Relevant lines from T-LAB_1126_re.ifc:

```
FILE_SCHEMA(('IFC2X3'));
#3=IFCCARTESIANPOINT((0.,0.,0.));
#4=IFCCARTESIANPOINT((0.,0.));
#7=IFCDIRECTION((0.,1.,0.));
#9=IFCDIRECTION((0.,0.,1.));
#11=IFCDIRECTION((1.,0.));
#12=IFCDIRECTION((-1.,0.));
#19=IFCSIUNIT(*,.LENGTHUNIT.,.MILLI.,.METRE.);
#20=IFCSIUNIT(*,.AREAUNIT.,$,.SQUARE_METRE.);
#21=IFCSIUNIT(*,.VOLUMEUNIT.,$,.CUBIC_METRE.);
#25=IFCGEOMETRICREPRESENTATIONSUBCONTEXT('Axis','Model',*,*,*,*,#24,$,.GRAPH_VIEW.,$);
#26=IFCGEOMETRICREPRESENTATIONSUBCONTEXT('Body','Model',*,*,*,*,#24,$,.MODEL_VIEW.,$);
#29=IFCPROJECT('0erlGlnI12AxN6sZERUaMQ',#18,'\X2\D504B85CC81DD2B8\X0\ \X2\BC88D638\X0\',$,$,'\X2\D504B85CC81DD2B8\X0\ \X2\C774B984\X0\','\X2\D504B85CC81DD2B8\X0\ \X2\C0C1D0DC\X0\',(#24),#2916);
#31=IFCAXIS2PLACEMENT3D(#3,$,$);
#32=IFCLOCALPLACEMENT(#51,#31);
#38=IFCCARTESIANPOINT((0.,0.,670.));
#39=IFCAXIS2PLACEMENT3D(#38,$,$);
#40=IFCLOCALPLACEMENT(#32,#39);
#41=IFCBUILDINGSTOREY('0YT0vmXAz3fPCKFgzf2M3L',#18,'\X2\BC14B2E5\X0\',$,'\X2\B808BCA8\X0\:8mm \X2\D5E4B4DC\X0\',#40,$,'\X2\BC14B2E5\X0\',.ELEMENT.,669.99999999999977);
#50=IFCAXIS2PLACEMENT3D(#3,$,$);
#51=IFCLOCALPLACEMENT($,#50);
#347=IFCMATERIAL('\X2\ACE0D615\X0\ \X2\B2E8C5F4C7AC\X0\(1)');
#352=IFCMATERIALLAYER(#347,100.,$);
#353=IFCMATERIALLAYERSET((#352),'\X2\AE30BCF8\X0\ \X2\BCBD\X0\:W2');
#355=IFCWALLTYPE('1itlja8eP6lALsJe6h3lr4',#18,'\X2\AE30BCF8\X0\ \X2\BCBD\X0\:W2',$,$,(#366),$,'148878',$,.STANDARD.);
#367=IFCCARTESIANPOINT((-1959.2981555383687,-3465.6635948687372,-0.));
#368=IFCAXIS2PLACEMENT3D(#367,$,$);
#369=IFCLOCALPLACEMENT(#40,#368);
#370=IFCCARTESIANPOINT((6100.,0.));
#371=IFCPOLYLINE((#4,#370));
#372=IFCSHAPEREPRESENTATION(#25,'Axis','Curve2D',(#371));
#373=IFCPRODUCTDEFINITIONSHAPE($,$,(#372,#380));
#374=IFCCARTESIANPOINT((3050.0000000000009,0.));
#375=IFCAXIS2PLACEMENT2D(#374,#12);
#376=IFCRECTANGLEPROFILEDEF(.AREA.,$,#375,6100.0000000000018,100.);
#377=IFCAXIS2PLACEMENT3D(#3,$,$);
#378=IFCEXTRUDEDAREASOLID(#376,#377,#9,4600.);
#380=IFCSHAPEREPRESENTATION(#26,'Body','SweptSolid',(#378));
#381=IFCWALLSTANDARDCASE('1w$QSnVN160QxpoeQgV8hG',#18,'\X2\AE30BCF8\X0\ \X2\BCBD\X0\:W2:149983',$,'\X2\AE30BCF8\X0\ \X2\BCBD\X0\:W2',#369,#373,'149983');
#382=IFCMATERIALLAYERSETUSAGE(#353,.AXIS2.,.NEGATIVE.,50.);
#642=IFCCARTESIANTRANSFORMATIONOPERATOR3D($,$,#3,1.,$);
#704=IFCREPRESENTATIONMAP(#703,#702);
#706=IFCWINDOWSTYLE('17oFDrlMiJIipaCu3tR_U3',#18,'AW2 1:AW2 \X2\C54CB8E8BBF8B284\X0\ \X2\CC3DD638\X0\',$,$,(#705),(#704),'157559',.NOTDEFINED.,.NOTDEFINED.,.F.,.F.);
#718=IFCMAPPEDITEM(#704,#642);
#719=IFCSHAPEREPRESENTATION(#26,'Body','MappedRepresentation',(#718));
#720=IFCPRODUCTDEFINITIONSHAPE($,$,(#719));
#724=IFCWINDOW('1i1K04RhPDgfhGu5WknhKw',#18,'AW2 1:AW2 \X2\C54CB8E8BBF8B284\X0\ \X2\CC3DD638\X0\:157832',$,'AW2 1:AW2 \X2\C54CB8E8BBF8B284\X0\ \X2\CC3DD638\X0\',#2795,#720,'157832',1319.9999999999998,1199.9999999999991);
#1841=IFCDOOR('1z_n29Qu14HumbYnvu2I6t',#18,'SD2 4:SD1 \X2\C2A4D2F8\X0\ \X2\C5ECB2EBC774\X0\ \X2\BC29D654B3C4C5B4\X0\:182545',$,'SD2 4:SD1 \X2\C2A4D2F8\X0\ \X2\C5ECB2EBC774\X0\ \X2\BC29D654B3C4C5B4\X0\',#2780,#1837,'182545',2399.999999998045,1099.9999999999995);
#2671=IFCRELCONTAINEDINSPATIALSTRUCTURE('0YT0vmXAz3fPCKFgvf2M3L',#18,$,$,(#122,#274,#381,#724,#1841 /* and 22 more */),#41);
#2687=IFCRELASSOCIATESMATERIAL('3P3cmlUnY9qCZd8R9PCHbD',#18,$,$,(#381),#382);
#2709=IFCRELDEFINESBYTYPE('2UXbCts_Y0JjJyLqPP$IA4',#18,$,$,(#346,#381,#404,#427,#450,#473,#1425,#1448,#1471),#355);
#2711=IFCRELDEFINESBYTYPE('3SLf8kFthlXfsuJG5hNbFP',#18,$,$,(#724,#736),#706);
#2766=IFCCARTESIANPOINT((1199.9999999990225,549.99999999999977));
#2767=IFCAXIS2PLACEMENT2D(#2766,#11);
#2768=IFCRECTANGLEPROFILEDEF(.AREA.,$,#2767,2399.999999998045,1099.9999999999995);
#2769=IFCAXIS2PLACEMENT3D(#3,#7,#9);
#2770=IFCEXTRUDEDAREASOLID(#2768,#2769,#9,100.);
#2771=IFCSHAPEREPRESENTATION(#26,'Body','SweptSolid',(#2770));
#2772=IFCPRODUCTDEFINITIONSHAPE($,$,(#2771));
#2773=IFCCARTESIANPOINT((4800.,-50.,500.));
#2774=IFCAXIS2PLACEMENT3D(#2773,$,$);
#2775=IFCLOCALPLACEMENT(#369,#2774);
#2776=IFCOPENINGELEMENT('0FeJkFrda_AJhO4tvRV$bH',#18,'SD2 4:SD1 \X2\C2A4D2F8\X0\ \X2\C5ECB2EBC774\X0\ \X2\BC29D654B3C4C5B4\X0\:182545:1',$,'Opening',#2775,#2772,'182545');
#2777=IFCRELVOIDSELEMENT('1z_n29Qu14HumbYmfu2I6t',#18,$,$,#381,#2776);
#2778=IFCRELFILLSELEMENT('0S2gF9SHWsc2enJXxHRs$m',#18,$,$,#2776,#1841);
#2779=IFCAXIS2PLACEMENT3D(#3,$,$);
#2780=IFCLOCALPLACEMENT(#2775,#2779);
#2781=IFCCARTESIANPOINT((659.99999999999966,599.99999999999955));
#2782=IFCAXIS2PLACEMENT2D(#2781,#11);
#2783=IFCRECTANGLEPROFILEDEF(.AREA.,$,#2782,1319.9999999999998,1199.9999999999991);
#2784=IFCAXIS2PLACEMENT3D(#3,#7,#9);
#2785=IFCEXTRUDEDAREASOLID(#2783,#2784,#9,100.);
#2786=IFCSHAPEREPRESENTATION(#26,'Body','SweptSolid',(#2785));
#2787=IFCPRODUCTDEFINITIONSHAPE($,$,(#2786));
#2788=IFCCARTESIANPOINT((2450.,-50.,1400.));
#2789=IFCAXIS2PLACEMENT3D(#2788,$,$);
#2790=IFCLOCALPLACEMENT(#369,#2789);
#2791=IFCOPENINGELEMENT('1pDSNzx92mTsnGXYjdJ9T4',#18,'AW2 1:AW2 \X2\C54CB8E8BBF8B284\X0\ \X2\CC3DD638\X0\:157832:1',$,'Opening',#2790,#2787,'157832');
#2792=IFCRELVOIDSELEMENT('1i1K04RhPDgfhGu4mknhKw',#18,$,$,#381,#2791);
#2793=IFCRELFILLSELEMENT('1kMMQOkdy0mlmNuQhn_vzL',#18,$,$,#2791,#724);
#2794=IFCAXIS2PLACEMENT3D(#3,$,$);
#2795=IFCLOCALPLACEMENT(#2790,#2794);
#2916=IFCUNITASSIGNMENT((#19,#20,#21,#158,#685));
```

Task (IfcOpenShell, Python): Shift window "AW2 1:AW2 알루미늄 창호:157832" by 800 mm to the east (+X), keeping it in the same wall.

```python
import ifcopenshell
import ifcopenshell.api.geometry
import ifcopenshell.util.placement
import ifcopenshell.util.unit

model = ifcopenshell.open("T-LAB_1126_re.ifc")
unit_scale = ifcopenshell.util.unit.calculate_unit_scale(model)

window = model.by_guid("1i1K04RhPDgfhGu5WknhKw")
opening = window.FillsVoids[0].RelatingOpeningElement
wall = opening.VoidsElements[0].RelatingBuildingElement

wall_matrix = ifcopenshell.util.placement.get_local_placement(wall.ObjectPlacement)
shift = wall_matrix[:3, 0] * 0.8 / unit_scale
before = ifcopenshell.util.placement.get_local_placement(window.ObjectPlacement)[:3, 3].copy()

# The window is placed relative to its opening, so it follows when the opening moves.
matrix = ifcopenshell.util.placement.get_local_placement(opening.ObjectPlacement)
matrix[:3, 3] += shift
ifcopenshell.api.geometry.edit_object_placement(
    model, product=opening, matrix=matrix, is_si=False, should_transform_children=True
)

after = ifcopenshell.util.placement.get_local_placement(window.ObjectPlacement)[:3, 3]
print("window moved by", (after - before).round(3) + 0.0)

model.write("T-LAB_1126_re_rev.ifc")
```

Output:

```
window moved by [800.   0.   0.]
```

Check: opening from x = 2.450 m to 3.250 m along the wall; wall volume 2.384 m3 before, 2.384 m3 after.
